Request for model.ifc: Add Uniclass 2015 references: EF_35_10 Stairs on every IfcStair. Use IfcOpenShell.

First a look at what the model holds.

```python
import ifcopenshell

model = ifcopenshell.open("model.ifc")
print(model.schema)
print("classifications:", [c.Name for c in model.by_type("IfcClassification")])
for ifc_class in ("IfcDoor", "IfcRoof", "IfcStair", "IfcWall", "IfcWindow"):
    print(ifc_class, len(model.by_type(ifc_class)))
```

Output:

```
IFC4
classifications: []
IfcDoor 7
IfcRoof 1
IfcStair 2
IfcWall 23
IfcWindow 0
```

```python
import ifcopenshell
import ifcopenshell.api.classification

model = ifcopenshell.open("model.ifc")

system = ifcopenshell.api.classification.add_classification(model, classification="Uniclass 2015")

codes = {
    "IfcStair": ("EF_35_10", "Stairs"),
}
for ifc_class, (code, name) in codes.items():
    products = model.by_type(ifc_class)
    ifcopenshell.api.classification.add_reference(
        model, products=products, classification=system, identification=code, name=name
    )
    print(code, len(products))

model.write("model_v2.ifc")
```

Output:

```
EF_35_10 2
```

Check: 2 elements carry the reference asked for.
